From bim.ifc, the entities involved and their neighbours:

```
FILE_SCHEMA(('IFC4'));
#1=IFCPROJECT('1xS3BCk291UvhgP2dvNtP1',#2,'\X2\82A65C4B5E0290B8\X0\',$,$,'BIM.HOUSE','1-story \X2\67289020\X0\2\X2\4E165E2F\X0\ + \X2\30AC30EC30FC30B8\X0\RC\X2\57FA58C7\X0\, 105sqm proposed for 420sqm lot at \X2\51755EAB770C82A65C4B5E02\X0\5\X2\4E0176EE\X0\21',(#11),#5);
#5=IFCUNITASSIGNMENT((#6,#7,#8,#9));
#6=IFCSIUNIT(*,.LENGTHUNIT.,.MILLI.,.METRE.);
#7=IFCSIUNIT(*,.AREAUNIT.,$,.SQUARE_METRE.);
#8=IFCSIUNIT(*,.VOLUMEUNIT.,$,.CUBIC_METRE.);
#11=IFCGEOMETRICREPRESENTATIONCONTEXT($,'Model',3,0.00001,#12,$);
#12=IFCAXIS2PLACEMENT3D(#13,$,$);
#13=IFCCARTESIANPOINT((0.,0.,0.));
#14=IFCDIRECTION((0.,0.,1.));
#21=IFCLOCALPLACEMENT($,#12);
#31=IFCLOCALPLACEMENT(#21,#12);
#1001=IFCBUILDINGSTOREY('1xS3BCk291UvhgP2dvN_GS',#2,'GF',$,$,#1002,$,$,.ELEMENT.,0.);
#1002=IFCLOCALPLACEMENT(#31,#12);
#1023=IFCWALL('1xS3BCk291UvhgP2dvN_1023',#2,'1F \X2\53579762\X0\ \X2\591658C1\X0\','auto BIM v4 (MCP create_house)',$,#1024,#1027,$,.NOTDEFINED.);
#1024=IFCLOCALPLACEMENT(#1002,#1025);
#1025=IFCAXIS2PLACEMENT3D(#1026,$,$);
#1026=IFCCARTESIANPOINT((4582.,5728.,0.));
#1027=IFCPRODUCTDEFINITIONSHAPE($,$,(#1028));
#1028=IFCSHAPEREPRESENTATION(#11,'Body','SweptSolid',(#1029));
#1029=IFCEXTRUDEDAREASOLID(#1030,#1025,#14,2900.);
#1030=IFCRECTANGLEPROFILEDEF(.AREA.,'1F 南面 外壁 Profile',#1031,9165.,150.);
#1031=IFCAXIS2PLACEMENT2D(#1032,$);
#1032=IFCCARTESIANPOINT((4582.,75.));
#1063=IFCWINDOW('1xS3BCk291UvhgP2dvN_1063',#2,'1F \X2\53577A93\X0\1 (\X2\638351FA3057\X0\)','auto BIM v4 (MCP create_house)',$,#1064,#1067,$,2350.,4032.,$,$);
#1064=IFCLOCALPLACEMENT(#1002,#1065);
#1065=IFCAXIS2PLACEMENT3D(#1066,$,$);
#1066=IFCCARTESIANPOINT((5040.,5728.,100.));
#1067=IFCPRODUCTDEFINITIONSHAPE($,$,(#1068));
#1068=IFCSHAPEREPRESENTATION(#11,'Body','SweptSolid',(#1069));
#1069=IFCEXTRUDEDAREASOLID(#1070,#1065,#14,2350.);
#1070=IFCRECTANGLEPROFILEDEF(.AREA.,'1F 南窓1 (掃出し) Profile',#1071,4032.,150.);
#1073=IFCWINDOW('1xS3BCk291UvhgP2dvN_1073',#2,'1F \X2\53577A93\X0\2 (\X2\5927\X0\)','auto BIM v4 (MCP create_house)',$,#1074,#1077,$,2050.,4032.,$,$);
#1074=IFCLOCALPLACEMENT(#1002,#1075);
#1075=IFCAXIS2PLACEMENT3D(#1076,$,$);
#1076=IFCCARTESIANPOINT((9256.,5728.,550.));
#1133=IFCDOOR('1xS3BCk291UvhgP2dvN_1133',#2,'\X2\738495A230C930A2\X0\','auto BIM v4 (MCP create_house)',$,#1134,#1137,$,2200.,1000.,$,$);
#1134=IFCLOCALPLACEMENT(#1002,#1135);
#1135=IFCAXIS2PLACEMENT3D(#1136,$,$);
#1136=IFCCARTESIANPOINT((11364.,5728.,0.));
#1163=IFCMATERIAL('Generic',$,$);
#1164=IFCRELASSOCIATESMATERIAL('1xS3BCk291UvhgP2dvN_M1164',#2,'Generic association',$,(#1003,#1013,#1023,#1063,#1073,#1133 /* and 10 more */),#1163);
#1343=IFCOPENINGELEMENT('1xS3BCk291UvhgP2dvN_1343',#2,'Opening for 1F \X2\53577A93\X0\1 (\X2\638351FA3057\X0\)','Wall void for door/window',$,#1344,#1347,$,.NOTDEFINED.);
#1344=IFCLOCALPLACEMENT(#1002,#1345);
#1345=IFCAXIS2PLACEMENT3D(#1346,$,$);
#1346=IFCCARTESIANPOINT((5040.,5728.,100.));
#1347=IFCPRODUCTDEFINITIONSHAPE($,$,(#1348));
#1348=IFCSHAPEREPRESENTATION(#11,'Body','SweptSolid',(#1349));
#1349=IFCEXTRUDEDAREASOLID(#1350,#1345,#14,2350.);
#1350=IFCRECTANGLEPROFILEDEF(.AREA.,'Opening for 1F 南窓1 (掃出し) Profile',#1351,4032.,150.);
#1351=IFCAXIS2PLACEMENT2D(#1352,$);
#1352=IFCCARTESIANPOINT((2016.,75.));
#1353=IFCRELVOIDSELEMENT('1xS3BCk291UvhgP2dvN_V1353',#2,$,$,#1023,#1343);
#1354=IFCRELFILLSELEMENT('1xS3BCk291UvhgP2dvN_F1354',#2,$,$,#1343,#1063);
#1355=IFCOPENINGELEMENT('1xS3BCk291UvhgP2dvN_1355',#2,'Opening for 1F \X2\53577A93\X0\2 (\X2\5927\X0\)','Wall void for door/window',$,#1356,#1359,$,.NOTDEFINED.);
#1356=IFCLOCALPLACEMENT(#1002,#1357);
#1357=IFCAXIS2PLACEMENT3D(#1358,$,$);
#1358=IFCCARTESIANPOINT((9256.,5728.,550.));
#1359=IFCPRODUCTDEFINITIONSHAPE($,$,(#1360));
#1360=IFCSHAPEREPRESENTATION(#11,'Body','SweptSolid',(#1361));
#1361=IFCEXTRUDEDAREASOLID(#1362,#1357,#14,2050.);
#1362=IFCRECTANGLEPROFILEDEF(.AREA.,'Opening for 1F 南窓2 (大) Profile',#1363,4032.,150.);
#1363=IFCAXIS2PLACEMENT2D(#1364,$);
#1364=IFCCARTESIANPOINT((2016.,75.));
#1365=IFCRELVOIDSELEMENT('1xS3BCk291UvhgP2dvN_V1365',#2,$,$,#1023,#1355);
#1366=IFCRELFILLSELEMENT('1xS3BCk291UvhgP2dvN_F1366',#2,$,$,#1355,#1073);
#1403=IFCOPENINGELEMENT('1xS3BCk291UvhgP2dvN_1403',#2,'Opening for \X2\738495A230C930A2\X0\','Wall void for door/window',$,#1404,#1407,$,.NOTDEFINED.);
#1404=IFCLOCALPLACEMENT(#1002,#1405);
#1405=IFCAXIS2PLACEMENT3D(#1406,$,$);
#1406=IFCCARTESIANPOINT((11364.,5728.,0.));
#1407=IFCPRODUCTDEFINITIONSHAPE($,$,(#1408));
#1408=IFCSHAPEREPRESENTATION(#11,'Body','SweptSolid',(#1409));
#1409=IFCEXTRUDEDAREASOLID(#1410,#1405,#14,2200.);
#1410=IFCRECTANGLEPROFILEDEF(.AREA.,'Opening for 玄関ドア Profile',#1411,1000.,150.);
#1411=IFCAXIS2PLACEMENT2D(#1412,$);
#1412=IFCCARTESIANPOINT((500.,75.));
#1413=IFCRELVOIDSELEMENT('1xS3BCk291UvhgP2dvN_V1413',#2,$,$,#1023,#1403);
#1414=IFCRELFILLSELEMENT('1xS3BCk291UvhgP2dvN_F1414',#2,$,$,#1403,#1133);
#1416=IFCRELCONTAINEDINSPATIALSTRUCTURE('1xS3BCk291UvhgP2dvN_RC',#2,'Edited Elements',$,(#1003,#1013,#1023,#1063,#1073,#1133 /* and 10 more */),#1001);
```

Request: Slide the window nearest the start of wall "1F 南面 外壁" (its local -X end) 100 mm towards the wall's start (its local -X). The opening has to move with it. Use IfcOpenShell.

```python
import ifcopenshell
import ifcopenshell.api.geometry
import ifcopenshell.util.placement
import ifcopenshell.util.unit

model = ifcopenshell.open("bim.ifc")
unit_scale = ifcopenshell.util.unit.calculate_unit_scale(model)

window = model.by_id(1063)
opening = window.FillsVoids[0].RelatingOpeningElement
wall = opening.VoidsElements[0].RelatingBuildingElement

wall_matrix = ifcopenshell.util.placement.get_local_placement(wall.ObjectPlacement)
shift = wall_matrix[:3, 0] * -0.1 / unit_scale
before = ifcopenshell.util.placement.get_local_placement(window.ObjectPlacement)[:3, 3].copy()

# The window is not placed relative to its opening, so move both.
for product in (opening, window):
    matrix = ifcopenshell.util.placement.get_local_placement(product.ObjectPlacement)
    matrix[:3, 3] += shift
    ifcopenshell.api.geometry.edit_object_placement(model, product=product, matrix=matrix, is_si=False)

after = ifcopenshell.util.placement.get_local_placement(window.ObjectPlacement)[:3, 3]
print("window moved by", (after - before).round(3) + 0.0)

model.write("bim_updated.ifc")
```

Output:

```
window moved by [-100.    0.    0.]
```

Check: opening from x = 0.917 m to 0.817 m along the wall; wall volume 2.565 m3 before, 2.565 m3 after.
